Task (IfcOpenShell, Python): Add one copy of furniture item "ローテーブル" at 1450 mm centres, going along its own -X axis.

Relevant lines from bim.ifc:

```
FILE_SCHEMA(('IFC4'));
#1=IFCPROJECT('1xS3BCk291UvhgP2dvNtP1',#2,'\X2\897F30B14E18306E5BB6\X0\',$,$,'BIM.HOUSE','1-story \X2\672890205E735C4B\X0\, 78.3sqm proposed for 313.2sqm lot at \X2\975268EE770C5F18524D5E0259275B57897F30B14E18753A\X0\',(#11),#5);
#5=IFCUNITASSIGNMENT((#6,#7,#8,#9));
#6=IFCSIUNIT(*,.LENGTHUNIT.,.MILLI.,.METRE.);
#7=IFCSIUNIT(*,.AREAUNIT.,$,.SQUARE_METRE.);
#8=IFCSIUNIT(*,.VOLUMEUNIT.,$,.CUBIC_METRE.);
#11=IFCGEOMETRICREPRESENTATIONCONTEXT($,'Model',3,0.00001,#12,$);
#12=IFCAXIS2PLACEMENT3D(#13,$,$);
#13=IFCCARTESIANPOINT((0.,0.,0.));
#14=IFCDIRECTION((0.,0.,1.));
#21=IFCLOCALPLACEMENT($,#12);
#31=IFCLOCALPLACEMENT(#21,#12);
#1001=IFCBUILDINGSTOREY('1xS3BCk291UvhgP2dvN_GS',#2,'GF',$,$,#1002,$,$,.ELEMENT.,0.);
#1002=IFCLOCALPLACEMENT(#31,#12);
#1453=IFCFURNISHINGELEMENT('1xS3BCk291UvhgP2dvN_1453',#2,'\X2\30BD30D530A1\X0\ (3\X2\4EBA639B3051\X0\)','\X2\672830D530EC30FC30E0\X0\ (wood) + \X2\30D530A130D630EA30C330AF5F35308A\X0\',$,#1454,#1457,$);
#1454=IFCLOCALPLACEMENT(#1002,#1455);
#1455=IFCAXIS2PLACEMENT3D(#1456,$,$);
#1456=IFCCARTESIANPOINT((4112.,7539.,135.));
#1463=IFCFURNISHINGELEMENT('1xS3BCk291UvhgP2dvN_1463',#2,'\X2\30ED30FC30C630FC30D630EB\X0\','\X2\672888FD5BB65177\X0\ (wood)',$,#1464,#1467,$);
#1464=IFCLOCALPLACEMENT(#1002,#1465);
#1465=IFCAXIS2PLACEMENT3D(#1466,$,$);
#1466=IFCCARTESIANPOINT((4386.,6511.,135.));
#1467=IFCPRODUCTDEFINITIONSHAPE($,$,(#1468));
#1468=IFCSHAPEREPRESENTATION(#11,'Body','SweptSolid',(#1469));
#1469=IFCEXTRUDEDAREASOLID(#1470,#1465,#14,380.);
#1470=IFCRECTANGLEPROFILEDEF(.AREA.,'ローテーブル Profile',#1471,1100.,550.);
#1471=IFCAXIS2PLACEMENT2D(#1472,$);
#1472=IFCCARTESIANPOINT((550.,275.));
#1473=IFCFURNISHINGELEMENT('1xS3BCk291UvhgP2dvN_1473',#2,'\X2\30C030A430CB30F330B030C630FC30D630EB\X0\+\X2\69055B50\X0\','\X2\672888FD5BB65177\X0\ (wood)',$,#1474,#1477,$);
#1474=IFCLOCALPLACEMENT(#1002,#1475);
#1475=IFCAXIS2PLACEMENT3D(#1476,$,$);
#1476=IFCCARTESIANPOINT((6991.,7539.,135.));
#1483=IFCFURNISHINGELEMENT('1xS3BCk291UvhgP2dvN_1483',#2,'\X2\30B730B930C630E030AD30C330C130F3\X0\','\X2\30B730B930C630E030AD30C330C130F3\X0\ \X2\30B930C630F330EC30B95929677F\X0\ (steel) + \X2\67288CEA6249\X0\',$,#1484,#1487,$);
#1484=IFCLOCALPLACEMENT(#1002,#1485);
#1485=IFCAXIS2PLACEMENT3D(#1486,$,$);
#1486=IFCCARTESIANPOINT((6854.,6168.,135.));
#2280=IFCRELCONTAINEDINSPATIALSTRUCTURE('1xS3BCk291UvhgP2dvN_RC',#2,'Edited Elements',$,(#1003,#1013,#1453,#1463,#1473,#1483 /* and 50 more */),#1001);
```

```python
import ifcopenshell
import ifcopenshell.api.geometry
import ifcopenshell.api.root
import ifcopenshell.util.element
import ifcopenshell.util.placement

model = ifcopenshell.open("bim.ifc")


def reuse_history(source, copy):
    """copy_class also copies each property set's owner history, people and application; keep the originals."""
    for rel in copy.IsDefinedBy:
        if rel.is_a("IfcRelDefinesByProperties") and (history := rel.RelatingPropertyDefinition.OwnerHistory):
            rel.RelatingPropertyDefinition.OwnerHistory = source.OwnerHistory
            ifcopenshell.util.element.remove_deep2(model, history)


source = model.by_guid("1xS3BCk291UvhgP2dvN_1463")
base = ifcopenshell.util.placement.get_local_placement(source.ObjectPlacement)
step = -base[:3, 0] * 1450.0

for i in range(1, 2):
    copy = ifcopenshell.api.root.copy_class(model, product=source)
    copy.Representation = ifcopenshell.util.element.copy_deep(
        model, source.Representation, exclude=["IfcGeometricRepresentationContext", "IfcRepresentationMap"]
    )
    reuse_history(source, copy)
    matrix = base.copy()
    matrix[:3, 3] += i * step
    print("added at", matrix[:3, 3].round(3) + 0.0)
    ifcopenshell.api.geometry.edit_object_placement(model, product=copy, matrix=matrix, is_si=False)

model.write("bim-out.ifc")
```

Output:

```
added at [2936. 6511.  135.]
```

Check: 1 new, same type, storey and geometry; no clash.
